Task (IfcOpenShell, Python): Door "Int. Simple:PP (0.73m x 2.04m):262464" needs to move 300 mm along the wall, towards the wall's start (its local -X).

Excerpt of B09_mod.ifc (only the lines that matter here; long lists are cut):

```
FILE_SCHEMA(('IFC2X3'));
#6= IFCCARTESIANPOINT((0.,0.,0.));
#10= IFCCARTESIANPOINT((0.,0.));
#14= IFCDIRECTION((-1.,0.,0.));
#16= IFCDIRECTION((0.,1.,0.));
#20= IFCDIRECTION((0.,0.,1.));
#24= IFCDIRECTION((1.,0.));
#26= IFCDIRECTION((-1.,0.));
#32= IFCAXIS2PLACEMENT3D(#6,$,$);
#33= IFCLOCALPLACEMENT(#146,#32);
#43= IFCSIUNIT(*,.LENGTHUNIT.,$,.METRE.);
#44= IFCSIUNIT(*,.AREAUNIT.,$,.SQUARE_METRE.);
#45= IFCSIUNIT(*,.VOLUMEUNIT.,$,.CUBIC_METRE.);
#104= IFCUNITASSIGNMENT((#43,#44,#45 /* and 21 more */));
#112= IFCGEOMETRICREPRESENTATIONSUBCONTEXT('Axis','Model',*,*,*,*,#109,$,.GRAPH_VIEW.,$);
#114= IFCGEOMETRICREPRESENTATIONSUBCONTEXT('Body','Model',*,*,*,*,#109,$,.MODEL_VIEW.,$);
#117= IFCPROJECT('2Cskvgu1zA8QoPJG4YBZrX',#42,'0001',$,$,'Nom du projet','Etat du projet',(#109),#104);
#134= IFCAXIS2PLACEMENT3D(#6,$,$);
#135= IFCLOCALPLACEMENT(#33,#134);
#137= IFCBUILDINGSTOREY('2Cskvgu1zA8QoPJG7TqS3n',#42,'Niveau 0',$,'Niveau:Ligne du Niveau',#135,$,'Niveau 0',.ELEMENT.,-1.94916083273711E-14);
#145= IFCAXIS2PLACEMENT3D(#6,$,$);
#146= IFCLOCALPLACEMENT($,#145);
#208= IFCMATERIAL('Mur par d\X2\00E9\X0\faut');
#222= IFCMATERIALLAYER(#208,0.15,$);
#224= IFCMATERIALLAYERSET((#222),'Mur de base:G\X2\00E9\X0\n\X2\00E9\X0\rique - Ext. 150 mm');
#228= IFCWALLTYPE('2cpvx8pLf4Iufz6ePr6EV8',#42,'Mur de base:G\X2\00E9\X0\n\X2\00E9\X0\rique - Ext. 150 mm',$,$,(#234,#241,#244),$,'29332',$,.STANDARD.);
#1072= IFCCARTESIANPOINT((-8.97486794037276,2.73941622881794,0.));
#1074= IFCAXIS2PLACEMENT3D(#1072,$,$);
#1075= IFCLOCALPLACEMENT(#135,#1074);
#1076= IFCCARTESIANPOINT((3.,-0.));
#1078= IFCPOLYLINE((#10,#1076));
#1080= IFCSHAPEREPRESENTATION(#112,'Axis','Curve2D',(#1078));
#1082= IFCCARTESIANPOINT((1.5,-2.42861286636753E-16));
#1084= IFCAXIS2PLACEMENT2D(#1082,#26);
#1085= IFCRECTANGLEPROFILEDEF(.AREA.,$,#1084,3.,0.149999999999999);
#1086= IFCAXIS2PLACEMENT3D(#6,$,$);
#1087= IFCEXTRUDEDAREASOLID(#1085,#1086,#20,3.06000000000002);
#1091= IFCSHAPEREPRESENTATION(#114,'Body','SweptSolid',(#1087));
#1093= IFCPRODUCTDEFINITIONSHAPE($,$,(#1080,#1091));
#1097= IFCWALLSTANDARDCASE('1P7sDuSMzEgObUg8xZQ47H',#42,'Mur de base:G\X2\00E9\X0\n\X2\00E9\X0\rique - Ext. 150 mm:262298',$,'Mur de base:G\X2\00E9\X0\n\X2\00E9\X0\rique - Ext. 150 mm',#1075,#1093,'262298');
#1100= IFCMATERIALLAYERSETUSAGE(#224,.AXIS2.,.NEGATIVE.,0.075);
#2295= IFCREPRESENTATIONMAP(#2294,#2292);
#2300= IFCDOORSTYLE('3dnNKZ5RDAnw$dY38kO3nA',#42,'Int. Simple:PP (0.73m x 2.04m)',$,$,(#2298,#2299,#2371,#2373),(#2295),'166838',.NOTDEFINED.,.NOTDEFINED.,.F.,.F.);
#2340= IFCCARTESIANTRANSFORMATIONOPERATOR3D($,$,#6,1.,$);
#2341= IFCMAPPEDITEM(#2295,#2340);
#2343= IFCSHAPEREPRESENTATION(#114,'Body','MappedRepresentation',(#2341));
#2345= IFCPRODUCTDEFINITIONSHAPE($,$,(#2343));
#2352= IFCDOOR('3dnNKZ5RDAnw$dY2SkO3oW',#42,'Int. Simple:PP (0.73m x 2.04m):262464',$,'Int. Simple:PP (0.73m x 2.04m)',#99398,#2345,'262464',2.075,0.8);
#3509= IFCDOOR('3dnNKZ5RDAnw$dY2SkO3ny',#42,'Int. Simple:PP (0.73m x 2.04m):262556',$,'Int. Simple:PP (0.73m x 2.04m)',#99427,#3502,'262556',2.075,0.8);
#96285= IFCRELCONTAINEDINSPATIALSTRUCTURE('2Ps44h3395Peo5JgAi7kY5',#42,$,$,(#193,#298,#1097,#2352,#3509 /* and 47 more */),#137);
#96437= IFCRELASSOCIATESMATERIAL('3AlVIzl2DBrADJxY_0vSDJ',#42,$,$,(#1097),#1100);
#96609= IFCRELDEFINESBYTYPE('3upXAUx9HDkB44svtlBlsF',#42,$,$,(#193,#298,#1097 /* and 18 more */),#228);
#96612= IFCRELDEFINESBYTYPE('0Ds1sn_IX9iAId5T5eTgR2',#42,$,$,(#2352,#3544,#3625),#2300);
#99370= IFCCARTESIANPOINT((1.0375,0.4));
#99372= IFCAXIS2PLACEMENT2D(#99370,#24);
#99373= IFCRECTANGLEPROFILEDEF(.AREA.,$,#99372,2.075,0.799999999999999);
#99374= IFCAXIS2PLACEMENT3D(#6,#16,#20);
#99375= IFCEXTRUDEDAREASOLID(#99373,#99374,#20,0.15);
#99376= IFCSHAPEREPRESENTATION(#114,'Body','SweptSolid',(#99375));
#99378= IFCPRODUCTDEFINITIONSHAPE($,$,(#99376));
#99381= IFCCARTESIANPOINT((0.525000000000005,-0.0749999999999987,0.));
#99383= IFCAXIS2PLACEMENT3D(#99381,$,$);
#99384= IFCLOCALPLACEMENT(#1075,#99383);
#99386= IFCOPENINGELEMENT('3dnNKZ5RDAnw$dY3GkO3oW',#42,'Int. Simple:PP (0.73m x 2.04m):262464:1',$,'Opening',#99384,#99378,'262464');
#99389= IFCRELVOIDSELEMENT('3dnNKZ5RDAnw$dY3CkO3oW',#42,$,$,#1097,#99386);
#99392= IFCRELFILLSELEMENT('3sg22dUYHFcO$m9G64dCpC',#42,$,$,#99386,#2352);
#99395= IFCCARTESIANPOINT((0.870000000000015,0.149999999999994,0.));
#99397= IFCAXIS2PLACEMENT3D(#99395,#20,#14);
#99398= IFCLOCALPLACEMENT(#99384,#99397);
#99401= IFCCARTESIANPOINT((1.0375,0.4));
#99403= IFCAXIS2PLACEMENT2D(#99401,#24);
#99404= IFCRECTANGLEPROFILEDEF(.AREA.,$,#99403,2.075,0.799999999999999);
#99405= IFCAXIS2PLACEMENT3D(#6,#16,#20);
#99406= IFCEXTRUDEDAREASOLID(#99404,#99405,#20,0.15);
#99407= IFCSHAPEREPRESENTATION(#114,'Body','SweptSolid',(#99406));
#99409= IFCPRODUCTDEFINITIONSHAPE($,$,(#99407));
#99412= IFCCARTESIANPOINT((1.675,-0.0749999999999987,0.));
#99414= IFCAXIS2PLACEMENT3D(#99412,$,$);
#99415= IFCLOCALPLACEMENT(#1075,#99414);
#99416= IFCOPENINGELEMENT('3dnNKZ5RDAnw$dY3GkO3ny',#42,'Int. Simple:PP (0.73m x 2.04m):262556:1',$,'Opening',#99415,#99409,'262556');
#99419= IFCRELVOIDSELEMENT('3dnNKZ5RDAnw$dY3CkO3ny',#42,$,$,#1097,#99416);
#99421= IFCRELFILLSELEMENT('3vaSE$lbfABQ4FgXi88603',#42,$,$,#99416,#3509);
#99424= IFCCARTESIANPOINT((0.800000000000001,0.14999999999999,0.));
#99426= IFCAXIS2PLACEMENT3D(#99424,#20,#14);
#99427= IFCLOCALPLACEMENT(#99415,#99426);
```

```python
import ifcopenshell
import ifcopenshell.api.geometry
import ifcopenshell.util.placement
import ifcopenshell.util.unit

model = ifcopenshell.open("B09_mod.ifc")
unit_scale = ifcopenshell.util.unit.calculate_unit_scale(model)

door = model.by_guid("3dnNKZ5RDAnw$dY2SkO3oW")
opening = door.FillsVoids[0].RelatingOpeningElement
wall = opening.VoidsElements[0].RelatingBuildingElement

wall_matrix = ifcopenshell.util.placement.get_local_placement(wall.ObjectPlacement)
shift = wall_matrix[:3, 0] * -0.3 / unit_scale
before = ifcopenshell.util.placement.get_local_placement(door.ObjectPlacement)[:3, 3].copy()

# The door is placed relative to its opening, so it follows when the opening moves.
matrix = ifcopenshell.util.placement.get_local_placement(opening.ObjectPlacement)
matrix[:3, 3] += shift
ifcopenshell.api.geometry.edit_object_placement(
    model, product=opening, matrix=matrix, is_si=False, should_transform_children=True
)

after = ifcopenshell.util.placement.get_local_placement(door.ObjectPlacement)[:3, 3]
print("door moved by", (after - before).round(3) + 0.0)

model.write("B09_mod_edited.ifc")
```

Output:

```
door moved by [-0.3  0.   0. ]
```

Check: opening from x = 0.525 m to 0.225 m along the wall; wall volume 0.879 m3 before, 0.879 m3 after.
